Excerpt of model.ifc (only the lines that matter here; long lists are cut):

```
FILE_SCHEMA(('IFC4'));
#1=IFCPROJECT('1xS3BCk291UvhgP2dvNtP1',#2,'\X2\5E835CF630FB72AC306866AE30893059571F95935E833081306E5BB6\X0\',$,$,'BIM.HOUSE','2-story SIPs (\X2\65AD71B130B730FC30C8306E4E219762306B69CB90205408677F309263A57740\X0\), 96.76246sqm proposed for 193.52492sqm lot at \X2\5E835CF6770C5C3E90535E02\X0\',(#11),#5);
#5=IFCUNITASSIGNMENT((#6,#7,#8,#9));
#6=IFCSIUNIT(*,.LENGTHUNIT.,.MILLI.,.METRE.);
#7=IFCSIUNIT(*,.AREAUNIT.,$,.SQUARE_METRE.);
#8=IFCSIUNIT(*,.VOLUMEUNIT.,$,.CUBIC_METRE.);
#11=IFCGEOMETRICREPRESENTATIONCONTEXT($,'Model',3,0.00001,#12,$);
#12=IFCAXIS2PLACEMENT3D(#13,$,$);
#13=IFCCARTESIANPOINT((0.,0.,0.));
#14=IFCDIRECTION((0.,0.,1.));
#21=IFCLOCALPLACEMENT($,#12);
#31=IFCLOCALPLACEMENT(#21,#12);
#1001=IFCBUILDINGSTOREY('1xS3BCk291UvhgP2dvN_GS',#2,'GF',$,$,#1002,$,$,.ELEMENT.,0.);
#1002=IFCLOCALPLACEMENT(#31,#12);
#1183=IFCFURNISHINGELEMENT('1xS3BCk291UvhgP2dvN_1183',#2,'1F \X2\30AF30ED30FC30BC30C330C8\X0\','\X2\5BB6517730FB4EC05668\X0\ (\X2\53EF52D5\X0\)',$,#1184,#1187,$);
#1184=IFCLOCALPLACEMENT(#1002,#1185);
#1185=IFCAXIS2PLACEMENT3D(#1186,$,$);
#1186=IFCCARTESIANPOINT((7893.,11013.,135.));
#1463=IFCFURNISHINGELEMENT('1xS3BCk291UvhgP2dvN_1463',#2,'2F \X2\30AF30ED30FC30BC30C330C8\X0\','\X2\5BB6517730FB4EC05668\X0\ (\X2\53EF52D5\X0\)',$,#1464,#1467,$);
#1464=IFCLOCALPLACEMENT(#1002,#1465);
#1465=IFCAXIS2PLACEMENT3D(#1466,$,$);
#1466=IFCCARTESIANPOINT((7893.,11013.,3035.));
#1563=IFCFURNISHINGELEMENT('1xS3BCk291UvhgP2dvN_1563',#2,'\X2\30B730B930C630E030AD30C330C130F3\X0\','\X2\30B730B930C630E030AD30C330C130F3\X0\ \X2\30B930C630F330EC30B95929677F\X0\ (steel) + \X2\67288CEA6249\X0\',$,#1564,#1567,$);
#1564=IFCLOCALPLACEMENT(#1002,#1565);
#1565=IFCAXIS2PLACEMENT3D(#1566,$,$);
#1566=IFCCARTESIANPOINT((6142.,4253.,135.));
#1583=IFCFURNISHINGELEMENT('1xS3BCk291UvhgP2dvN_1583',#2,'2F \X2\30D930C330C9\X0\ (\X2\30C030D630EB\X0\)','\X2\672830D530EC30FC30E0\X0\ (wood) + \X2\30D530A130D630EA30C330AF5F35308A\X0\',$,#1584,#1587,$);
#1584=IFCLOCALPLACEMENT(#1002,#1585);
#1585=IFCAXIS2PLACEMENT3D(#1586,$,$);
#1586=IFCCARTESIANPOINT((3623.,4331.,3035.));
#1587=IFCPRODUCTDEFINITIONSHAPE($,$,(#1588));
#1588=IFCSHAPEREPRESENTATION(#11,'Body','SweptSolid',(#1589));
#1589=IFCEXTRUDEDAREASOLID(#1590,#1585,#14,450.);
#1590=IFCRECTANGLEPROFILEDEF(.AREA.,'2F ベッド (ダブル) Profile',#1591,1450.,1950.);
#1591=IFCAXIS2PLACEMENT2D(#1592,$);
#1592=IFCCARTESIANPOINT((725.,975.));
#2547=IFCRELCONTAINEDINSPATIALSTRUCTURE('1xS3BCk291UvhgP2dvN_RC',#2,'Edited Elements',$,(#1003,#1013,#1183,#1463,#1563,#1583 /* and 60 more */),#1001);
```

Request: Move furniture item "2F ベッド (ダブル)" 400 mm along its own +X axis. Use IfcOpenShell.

```python
import ifcopenshell
import ifcopenshell.api.geometry
import ifcopenshell.util.placement

model = ifcopenshell.open("model.ifc")

item = model.by_guid("1xS3BCk291UvhgP2dvN_1583")
matrix = ifcopenshell.util.placement.get_local_placement(item.ObjectPlacement)
matrix[:3, 3] += matrix[:3, 0] * 400.0
ifcopenshell.api.geometry.edit_object_placement(model, product=item, matrix=matrix, is_si=False)

print(ifcopenshell.util.placement.get_local_placement(item.ObjectPlacement).round(3) + 0.0)

model.write("model_v2.ifc")
```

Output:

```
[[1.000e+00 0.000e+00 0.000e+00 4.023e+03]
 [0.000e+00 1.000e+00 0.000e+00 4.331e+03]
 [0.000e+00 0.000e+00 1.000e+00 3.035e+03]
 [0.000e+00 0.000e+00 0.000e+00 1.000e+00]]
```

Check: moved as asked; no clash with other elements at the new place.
